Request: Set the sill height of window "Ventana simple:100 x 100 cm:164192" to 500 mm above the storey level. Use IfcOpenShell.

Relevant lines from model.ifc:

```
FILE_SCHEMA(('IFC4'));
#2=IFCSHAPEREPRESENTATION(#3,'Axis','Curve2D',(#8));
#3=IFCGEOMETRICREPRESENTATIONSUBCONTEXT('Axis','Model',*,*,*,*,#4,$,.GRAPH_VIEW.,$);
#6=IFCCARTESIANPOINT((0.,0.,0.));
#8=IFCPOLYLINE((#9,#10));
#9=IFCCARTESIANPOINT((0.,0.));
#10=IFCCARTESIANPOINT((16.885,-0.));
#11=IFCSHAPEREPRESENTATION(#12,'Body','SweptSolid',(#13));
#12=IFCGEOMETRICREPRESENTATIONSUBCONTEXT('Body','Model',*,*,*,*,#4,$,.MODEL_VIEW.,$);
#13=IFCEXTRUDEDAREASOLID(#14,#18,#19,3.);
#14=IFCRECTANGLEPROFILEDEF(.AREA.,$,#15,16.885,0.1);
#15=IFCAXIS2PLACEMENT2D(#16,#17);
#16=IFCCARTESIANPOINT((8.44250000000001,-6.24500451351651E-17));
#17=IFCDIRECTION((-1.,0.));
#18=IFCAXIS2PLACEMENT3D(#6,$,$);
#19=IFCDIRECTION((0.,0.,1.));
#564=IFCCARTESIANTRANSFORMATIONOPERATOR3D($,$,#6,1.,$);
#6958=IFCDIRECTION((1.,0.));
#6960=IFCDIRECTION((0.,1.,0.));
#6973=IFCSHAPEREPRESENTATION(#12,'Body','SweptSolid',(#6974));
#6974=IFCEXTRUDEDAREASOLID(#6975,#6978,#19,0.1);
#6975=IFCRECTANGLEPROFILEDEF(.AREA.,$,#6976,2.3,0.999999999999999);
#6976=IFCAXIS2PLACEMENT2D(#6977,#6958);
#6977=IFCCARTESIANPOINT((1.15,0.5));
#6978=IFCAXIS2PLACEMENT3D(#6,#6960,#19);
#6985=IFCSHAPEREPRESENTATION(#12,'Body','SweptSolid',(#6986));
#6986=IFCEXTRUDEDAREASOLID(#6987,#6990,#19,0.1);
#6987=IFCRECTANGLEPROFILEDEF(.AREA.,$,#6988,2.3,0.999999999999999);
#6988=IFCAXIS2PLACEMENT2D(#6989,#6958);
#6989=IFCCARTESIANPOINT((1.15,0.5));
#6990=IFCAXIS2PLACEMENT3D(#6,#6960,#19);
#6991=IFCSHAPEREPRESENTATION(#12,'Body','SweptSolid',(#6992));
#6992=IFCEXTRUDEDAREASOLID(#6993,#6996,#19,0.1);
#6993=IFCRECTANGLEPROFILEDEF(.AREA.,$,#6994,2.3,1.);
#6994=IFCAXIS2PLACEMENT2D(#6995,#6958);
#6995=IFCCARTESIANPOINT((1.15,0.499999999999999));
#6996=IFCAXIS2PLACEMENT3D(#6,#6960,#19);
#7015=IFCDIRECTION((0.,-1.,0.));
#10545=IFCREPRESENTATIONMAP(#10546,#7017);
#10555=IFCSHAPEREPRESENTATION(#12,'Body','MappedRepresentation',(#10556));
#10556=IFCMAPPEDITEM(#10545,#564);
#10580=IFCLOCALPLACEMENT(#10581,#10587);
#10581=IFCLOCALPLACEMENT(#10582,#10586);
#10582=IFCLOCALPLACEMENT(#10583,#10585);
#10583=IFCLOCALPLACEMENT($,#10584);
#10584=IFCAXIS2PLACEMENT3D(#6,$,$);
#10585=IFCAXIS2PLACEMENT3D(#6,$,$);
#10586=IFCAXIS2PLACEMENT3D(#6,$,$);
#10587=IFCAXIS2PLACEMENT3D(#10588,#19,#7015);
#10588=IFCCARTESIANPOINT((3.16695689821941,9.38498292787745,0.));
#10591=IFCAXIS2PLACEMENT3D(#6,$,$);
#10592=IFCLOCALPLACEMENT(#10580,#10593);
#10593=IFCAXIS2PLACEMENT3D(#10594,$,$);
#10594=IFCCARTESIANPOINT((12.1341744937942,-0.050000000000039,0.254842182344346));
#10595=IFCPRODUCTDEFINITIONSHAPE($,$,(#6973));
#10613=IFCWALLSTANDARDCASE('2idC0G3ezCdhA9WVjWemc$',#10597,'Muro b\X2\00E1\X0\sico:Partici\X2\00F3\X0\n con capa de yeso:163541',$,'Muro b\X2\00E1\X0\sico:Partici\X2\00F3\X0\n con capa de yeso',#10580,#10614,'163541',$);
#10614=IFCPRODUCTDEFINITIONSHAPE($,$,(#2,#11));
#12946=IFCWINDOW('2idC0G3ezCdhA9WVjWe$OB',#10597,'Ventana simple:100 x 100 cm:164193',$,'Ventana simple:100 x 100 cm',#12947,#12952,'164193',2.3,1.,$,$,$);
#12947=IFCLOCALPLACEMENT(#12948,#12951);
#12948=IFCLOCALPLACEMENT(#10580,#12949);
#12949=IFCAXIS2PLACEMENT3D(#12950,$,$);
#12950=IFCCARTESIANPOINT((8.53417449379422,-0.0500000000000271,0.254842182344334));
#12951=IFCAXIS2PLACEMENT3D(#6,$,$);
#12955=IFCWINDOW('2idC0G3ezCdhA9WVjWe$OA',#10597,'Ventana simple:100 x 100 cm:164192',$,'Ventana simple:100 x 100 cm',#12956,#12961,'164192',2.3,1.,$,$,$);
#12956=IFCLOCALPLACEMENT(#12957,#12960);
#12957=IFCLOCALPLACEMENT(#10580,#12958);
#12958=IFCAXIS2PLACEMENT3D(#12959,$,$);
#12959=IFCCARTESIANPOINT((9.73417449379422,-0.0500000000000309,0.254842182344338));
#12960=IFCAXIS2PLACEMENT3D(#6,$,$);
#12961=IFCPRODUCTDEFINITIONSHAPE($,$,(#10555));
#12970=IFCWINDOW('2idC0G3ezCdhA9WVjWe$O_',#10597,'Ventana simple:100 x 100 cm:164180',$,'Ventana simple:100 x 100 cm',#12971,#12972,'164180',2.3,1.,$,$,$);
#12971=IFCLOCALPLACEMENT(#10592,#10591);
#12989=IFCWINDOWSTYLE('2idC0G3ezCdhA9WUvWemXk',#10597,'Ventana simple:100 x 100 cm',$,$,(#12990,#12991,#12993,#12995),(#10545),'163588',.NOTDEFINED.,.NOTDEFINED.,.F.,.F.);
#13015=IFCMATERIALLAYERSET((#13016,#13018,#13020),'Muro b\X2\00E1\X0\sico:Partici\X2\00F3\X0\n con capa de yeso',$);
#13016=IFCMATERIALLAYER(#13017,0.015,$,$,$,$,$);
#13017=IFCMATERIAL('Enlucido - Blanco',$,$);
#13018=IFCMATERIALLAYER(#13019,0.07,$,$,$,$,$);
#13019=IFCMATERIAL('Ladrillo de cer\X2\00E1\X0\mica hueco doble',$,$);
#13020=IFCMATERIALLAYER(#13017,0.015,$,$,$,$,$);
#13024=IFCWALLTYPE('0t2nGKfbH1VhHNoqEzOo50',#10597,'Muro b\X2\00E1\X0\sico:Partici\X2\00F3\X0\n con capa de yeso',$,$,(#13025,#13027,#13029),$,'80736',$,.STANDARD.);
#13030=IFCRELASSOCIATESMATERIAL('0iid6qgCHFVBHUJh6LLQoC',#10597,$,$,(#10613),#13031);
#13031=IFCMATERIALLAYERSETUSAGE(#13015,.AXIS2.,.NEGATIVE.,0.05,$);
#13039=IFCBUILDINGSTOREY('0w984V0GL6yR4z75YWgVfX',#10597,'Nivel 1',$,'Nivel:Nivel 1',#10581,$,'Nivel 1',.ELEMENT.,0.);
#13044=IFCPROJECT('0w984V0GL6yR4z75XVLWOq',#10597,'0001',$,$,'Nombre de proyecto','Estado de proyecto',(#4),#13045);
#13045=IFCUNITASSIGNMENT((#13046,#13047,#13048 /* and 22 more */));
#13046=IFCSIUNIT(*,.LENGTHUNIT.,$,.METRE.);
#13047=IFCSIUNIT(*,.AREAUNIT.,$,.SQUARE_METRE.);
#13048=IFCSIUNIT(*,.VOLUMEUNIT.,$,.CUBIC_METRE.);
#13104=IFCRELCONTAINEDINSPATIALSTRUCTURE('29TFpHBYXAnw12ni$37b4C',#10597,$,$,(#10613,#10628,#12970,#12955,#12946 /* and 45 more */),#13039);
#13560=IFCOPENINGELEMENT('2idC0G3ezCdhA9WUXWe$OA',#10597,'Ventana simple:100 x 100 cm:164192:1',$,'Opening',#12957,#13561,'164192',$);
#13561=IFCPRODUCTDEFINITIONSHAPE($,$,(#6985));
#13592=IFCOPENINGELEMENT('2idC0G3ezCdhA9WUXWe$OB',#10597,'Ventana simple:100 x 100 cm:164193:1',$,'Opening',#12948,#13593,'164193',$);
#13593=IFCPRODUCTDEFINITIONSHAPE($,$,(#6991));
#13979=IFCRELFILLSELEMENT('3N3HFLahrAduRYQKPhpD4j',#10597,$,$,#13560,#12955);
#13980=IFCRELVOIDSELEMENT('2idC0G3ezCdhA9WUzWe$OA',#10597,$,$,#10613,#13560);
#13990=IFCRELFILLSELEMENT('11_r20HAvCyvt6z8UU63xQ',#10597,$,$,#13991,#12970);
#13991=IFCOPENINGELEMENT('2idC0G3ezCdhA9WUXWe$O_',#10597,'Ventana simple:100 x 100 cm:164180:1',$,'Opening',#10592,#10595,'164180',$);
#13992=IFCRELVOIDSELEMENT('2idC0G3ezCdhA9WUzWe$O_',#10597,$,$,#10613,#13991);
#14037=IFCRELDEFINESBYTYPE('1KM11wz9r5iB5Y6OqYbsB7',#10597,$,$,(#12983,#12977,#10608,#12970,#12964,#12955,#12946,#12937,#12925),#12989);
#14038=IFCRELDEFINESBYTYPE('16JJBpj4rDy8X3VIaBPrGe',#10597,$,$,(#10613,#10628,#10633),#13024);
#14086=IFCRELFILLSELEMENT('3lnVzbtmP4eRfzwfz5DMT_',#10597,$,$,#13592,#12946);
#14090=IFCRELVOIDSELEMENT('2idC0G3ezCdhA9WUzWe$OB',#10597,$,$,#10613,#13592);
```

```python
import numpy as np
import ifcopenshell
import ifcopenshell.api.geometry
import ifcopenshell.geom
import ifcopenshell.util.element
import ifcopenshell.util.placement
import ifcopenshell.util.shape
import ifcopenshell.util.unit

model = ifcopenshell.open("model.ifc")
unit_scale = ifcopenshell.util.unit.calculate_unit_scale(model)

window = model.by_guid("2idC0G3ezCdhA9WVjWe$OA")
opening = window.FillsVoids[0].RelatingOpeningElement
storey = ifcopenshell.util.element.get_container(window, ifc_class="IfcBuildingStorey")
level = ifcopenshell.util.placement.get_local_placement(storey.ObjectPlacement)[2, 3]

# The opening's origin need not be at the sill, so measure its lowest point.
shape = ifcopenshell.geom.create_shape(ifcopenshell.geom.settings(), opening)
bottom = ifcopenshell.util.shape.get_shape_bottom_elevation(shape, shape.geometry) / unit_scale
dz = level + 0.5 / unit_scale - bottom

shift = np.array([0.0, 0.0, dz])
# The window is placed relative to its opening, so it follows when the opening moves.
matrix = ifcopenshell.util.placement.get_local_placement(opening.ObjectPlacement)
matrix[:3, 3] += shift
ifcopenshell.api.geometry.edit_object_placement(
    model, product=opening, matrix=matrix, is_si=False, should_transform_children=True
)

print(f"moved by {dz * unit_scale:+.3f} m")

model.write("model_v2.ifc")
```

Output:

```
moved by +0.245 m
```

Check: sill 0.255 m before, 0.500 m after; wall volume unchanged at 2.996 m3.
